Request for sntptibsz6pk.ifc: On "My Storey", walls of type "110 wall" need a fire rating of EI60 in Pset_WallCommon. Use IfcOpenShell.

First a look at what the model holds.

```python
import ifcopenshell
import ifcopenshell.util.element

model = ifcopenshell.open("sntptibsz6pk.ifc")
print(model.schema)
storey = next(s for s in model.by_type("IfcBuildingStorey") if s.Name == "My Storey")
walls = [e for e in ifcopenshell.util.element.get_decomposition(storey) if e.is_a("IfcWall")]
seen = {}
for e in walls:
    element_type = ifcopenshell.util.element.get_type(e)
    key = (element_type.Name if element_type != e and element_type else None, ifcopenshell.util.element.get_pset(e, "Pset_WallCommon", "FireRating"))
    seen[key] = seen.get(key, 0) + 1
for (name, value), count in sorted(seen.items(), key=str):
    print(count, "x", name, "|", value)
```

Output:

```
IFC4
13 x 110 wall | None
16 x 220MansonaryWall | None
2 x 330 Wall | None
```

```python
import ifcopenshell
import ifcopenshell.api.pset
import ifcopenshell.util.element

model = ifcopenshell.open("sntptibsz6pk.ifc")

storey = next(s for s in model.by_type("IfcBuildingStorey") if s.Name == "My Storey")
walls = [e for e in ifcopenshell.util.element.get_decomposition(storey) if e.is_a("IfcWall")]

count = 0
for e in walls:
    element_type = ifcopenshell.util.element.get_type(e)
    if element_type in (None, e) or element_type.Name != "110 wall":
        continue
    # add_pset returns the element's existing set when there is one.
    pset = ifcopenshell.api.pset.add_pset(model, product=e, name="Pset_WallCommon")
    ifcopenshell.api.pset.edit_pset(model, pset=pset, properties={"FireRating": "EI60"})
    count += 1

print(count, "walls updated")

model.write("sntptibsz6pk-out.ifc")
```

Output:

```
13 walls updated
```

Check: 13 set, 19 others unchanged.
